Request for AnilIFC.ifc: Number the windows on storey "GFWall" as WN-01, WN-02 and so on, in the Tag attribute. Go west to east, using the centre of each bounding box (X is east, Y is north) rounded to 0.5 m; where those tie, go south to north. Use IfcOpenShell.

First a look at what the model holds.

```python
import ifcopenshell
import ifcopenshell.util.element
import ifcopenshell.util.placement

model = ifcopenshell.open("AnilIFC.ifc")
print(model.schema)
storey = next(s for s in model.by_type("IfcBuildingStorey") if s.Name == "GFWall")
windows = [e for e in ifcopenshell.util.element.get_decomposition(storey) if e.is_a("IfcWindow")]
for e in sorted(windows, key=lambda e: e.id()):
    origin = ifcopenshell.util.placement.get_local_placement(e.ObjectPlacement)[:3, 3]
    print(e.id(), e.Tag, e.Name, origin.round(2) + 0.0, sep=" | ")
```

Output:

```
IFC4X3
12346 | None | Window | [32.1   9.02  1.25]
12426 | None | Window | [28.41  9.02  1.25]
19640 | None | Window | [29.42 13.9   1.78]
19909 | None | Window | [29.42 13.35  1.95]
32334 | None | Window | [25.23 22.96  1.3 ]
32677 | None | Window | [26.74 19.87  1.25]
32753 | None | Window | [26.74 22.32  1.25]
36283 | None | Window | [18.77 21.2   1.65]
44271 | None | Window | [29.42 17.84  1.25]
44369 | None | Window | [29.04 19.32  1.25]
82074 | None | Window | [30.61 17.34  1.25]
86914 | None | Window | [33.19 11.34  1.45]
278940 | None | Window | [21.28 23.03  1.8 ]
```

```python
import ifcopenshell
import ifcopenshell.geom
import ifcopenshell.util.element
import ifcopenshell.util.shape

model = ifcopenshell.open("AnilIFC.ifc")
settings = ifcopenshell.geom.settings()
settings.set("use-world-coords", True)


def centre(element):
    shape = ifcopenshell.geom.create_shape(settings, element)
    return ifcopenshell.util.shape.get_bbox_centroid(shape.geometry)


storey = next(s for s in model.by_type("IfcBuildingStorey") if s.Name == "GFWall")
windows = [e for e in ifcopenshell.util.element.get_decomposition(storey) if e.is_a("IfcWindow")]

# Insertion points can sit at a corner or the storey origin, so sort by the geometry (in metres).
centres = {e: centre(e) for e in windows}
windows.sort(key=lambda e: (round(centres[e][0] / 0.5), centres[e][1]))

for i, e in enumerate(windows, start=1):
    number = f"WN-{i:02d}"
    e.Tag = number
    print(e.id(), number)

model.write("AnilIFC_v2.ifc")
```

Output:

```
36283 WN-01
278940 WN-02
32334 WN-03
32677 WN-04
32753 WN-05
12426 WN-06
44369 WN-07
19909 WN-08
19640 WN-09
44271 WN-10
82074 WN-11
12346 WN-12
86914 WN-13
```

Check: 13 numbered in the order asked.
